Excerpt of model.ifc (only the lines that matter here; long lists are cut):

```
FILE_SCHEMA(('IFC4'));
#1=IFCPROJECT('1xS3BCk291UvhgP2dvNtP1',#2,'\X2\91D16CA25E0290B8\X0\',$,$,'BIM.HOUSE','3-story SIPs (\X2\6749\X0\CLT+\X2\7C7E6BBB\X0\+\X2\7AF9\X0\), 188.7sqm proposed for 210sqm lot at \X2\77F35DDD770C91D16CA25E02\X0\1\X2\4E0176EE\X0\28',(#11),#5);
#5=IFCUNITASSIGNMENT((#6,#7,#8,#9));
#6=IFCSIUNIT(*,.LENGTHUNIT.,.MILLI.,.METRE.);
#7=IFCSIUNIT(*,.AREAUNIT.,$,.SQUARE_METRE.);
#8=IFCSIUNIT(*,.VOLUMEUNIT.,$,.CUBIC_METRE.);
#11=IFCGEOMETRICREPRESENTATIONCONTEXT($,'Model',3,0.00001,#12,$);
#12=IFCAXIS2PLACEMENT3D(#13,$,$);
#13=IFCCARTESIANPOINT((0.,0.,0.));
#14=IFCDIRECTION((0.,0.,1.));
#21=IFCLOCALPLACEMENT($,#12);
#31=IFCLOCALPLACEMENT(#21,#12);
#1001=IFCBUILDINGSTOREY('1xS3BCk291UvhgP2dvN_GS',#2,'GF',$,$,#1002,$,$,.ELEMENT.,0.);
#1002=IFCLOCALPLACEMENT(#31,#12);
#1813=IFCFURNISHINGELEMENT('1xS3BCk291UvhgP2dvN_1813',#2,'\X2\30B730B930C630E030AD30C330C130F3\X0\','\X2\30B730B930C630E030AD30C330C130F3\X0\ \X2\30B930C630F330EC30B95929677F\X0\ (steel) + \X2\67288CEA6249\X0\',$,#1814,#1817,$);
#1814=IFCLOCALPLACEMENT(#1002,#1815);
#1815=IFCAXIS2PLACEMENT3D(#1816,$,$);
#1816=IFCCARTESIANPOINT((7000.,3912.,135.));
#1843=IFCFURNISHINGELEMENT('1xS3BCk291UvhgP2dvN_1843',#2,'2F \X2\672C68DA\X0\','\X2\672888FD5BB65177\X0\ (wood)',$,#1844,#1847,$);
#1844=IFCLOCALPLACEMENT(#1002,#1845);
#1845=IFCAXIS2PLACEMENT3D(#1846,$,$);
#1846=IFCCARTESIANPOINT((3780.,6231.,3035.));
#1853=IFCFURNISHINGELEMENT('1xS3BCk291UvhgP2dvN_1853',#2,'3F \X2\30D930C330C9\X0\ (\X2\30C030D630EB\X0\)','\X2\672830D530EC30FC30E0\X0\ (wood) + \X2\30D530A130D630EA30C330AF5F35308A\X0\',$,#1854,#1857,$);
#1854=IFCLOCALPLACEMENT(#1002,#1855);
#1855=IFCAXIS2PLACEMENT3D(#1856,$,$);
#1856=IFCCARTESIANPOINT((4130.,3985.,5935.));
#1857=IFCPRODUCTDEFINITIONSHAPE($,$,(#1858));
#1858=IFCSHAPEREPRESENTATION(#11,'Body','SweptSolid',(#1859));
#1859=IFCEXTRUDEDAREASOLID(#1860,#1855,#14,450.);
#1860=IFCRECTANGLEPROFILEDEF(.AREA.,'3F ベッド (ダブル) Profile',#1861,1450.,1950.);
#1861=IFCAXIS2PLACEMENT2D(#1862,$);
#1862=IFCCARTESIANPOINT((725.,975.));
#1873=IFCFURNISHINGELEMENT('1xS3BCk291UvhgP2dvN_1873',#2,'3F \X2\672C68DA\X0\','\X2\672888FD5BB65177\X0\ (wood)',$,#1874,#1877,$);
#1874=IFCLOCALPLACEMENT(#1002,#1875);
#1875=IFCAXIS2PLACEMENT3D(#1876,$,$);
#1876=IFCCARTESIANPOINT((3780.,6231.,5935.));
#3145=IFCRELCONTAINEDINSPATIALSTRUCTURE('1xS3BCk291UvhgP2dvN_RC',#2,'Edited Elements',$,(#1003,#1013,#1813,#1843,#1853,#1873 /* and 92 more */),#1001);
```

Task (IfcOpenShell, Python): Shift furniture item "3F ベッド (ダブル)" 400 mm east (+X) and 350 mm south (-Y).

```python
import ifcopenshell
import ifcopenshell.api.geometry
import ifcopenshell.util.placement

model = ifcopenshell.open("model.ifc")

item = model.by_guid("1xS3BCk291UvhgP2dvN_1853")
matrix = ifcopenshell.util.placement.get_local_placement(item.ObjectPlacement)
matrix[0, 3] += 400.0
matrix[1, 3] -= 350.0
ifcopenshell.api.geometry.edit_object_placement(model, product=item, matrix=matrix, is_si=False)

print(ifcopenshell.util.placement.get_local_placement(item.ObjectPlacement).round(3) + 0.0)

model.write("model_rev.ifc")
```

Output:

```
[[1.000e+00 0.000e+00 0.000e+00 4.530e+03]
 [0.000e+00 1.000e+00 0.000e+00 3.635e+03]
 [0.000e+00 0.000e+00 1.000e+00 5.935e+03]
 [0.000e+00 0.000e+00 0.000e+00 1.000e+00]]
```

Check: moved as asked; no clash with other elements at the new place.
